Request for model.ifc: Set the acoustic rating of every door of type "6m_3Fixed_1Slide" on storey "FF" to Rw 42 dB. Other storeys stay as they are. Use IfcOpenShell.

First a look at what the model holds.

```python
import ifcopenshell
import ifcopenshell.util.element

model = ifcopenshell.open("model.ifc")
print(model.schema)
storey = next(s for s in model.by_type("IfcBuildingStorey") if s.Name == "FF")
doors = [e for e in ifcopenshell.util.element.get_decomposition(storey) if e.is_a("IfcDoor")]
seen = {}
for e in doors:
    element_type = ifcopenshell.util.element.get_type(e)
    key = (element_type.Name if element_type != e and element_type else None, ifcopenshell.util.element.get_pset(e, "Pset_DoorCommon", "AcousticRating"))
    seen[key] = seen.get(key, 0) + 1
for (name, value), count in sorted(seen.items(), key=str):
    print(count, "x", name, "|", value)
```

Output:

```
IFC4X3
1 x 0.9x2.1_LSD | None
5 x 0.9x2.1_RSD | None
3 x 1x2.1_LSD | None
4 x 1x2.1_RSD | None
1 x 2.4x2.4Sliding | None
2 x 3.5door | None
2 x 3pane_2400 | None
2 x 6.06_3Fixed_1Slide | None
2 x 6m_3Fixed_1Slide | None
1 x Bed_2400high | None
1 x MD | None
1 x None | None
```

```python
import ifcopenshell
import ifcopenshell.api.pset
import ifcopenshell.util.element

model = ifcopenshell.open("model.ifc")

storey = next(s for s in model.by_type("IfcBuildingStorey") if s.Name == "FF")
doors = [e for e in ifcopenshell.util.element.get_decomposition(storey) if e.is_a("IfcDoor")]

count = 0
for e in doors:
    element_type = ifcopenshell.util.element.get_type(e)
    if element_type in (None, e) or element_type.Name != "6m_3Fixed_1Slide":
        continue
    # add_pset returns the element's existing set when there is one.
    pset = ifcopenshell.api.pset.add_pset(model, product=e, name="Pset_DoorCommon")
    ifcopenshell.api.pset.edit_pset(model, pset=pset, properties={"AcousticRating": "Rw 42 dB"})
    count += 1

print(count, "doors updated")

model.write("model_updated.ifc")
```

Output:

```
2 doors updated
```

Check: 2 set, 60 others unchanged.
